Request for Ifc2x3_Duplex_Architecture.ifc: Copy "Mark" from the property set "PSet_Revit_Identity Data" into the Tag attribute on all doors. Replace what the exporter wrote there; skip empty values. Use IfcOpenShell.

First a look at what the model holds.

```python
import ifcopenshell
import ifcopenshell.util.element

model = ifcopenshell.open("Ifc2x3_Duplex_Architecture.ifc")
print(model.schema)
doors = model.by_type("IfcDoor")
print(len(doors), "doors")
for e in doors[:8]:
    source = ifcopenshell.util.element.get_pset(e, "PSet_Revit_Identity Data", "Mark")
    target = e.Tag
    print(e.id(), repr(source), repr(target), sep=" | ")
```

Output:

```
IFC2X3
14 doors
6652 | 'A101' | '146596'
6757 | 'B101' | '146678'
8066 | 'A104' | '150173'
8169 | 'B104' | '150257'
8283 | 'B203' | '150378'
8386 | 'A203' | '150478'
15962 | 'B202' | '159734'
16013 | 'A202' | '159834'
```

```python
import ifcopenshell
import ifcopenshell.util.element

model = ifcopenshell.open("Ifc2x3_Duplex_Architecture.ifc")

count = 0
for e in model.by_type("IfcDoor"):
    value = ifcopenshell.util.element.get_pset(e, "PSet_Revit_Identity Data", "Mark")
    current = e.Tag
    if not value or not value.strip() or current == value:
        continue
    e.Tag = value
    count += 1

print(count, "doors updated")

model.write("Ifc2x3_Duplex_Architecture_rev.ifc")
```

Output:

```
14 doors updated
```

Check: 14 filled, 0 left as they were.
